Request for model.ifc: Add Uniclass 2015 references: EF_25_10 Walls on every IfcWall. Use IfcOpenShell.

First a look at what the model holds.

```python
import ifcopenshell

model = ifcopenshell.open("model.ifc")
print(model.schema)
print("classifications:", [c.Name for c in model.by_type("IfcClassification")])
for ifc_class in ("IfcDoor", "IfcRoof", "IfcStair", "IfcWall", "IfcWindow"):
    print(ifc_class, len(model.by_type(ifc_class)))
```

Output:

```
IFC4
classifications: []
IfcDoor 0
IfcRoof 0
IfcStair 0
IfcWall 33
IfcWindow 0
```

```python
import ifcopenshell
import ifcopenshell.api.classification

model = ifcopenshell.open("model.ifc")

system = ifcopenshell.api.classification.add_classification(model, classification="Uniclass 2015")

codes = {
    "IfcWall": ("EF_25_10", "Walls"),
}
for ifc_class, (code, name) in codes.items():
    products = model.by_type(ifc_class)
    ifcopenshell.api.classification.add_reference(
        model, products=products, classification=system, identification=code, name=name
    )
    print(code, len(products))

model.write("model_edited.ifc")
```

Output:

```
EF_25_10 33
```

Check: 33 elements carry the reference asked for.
